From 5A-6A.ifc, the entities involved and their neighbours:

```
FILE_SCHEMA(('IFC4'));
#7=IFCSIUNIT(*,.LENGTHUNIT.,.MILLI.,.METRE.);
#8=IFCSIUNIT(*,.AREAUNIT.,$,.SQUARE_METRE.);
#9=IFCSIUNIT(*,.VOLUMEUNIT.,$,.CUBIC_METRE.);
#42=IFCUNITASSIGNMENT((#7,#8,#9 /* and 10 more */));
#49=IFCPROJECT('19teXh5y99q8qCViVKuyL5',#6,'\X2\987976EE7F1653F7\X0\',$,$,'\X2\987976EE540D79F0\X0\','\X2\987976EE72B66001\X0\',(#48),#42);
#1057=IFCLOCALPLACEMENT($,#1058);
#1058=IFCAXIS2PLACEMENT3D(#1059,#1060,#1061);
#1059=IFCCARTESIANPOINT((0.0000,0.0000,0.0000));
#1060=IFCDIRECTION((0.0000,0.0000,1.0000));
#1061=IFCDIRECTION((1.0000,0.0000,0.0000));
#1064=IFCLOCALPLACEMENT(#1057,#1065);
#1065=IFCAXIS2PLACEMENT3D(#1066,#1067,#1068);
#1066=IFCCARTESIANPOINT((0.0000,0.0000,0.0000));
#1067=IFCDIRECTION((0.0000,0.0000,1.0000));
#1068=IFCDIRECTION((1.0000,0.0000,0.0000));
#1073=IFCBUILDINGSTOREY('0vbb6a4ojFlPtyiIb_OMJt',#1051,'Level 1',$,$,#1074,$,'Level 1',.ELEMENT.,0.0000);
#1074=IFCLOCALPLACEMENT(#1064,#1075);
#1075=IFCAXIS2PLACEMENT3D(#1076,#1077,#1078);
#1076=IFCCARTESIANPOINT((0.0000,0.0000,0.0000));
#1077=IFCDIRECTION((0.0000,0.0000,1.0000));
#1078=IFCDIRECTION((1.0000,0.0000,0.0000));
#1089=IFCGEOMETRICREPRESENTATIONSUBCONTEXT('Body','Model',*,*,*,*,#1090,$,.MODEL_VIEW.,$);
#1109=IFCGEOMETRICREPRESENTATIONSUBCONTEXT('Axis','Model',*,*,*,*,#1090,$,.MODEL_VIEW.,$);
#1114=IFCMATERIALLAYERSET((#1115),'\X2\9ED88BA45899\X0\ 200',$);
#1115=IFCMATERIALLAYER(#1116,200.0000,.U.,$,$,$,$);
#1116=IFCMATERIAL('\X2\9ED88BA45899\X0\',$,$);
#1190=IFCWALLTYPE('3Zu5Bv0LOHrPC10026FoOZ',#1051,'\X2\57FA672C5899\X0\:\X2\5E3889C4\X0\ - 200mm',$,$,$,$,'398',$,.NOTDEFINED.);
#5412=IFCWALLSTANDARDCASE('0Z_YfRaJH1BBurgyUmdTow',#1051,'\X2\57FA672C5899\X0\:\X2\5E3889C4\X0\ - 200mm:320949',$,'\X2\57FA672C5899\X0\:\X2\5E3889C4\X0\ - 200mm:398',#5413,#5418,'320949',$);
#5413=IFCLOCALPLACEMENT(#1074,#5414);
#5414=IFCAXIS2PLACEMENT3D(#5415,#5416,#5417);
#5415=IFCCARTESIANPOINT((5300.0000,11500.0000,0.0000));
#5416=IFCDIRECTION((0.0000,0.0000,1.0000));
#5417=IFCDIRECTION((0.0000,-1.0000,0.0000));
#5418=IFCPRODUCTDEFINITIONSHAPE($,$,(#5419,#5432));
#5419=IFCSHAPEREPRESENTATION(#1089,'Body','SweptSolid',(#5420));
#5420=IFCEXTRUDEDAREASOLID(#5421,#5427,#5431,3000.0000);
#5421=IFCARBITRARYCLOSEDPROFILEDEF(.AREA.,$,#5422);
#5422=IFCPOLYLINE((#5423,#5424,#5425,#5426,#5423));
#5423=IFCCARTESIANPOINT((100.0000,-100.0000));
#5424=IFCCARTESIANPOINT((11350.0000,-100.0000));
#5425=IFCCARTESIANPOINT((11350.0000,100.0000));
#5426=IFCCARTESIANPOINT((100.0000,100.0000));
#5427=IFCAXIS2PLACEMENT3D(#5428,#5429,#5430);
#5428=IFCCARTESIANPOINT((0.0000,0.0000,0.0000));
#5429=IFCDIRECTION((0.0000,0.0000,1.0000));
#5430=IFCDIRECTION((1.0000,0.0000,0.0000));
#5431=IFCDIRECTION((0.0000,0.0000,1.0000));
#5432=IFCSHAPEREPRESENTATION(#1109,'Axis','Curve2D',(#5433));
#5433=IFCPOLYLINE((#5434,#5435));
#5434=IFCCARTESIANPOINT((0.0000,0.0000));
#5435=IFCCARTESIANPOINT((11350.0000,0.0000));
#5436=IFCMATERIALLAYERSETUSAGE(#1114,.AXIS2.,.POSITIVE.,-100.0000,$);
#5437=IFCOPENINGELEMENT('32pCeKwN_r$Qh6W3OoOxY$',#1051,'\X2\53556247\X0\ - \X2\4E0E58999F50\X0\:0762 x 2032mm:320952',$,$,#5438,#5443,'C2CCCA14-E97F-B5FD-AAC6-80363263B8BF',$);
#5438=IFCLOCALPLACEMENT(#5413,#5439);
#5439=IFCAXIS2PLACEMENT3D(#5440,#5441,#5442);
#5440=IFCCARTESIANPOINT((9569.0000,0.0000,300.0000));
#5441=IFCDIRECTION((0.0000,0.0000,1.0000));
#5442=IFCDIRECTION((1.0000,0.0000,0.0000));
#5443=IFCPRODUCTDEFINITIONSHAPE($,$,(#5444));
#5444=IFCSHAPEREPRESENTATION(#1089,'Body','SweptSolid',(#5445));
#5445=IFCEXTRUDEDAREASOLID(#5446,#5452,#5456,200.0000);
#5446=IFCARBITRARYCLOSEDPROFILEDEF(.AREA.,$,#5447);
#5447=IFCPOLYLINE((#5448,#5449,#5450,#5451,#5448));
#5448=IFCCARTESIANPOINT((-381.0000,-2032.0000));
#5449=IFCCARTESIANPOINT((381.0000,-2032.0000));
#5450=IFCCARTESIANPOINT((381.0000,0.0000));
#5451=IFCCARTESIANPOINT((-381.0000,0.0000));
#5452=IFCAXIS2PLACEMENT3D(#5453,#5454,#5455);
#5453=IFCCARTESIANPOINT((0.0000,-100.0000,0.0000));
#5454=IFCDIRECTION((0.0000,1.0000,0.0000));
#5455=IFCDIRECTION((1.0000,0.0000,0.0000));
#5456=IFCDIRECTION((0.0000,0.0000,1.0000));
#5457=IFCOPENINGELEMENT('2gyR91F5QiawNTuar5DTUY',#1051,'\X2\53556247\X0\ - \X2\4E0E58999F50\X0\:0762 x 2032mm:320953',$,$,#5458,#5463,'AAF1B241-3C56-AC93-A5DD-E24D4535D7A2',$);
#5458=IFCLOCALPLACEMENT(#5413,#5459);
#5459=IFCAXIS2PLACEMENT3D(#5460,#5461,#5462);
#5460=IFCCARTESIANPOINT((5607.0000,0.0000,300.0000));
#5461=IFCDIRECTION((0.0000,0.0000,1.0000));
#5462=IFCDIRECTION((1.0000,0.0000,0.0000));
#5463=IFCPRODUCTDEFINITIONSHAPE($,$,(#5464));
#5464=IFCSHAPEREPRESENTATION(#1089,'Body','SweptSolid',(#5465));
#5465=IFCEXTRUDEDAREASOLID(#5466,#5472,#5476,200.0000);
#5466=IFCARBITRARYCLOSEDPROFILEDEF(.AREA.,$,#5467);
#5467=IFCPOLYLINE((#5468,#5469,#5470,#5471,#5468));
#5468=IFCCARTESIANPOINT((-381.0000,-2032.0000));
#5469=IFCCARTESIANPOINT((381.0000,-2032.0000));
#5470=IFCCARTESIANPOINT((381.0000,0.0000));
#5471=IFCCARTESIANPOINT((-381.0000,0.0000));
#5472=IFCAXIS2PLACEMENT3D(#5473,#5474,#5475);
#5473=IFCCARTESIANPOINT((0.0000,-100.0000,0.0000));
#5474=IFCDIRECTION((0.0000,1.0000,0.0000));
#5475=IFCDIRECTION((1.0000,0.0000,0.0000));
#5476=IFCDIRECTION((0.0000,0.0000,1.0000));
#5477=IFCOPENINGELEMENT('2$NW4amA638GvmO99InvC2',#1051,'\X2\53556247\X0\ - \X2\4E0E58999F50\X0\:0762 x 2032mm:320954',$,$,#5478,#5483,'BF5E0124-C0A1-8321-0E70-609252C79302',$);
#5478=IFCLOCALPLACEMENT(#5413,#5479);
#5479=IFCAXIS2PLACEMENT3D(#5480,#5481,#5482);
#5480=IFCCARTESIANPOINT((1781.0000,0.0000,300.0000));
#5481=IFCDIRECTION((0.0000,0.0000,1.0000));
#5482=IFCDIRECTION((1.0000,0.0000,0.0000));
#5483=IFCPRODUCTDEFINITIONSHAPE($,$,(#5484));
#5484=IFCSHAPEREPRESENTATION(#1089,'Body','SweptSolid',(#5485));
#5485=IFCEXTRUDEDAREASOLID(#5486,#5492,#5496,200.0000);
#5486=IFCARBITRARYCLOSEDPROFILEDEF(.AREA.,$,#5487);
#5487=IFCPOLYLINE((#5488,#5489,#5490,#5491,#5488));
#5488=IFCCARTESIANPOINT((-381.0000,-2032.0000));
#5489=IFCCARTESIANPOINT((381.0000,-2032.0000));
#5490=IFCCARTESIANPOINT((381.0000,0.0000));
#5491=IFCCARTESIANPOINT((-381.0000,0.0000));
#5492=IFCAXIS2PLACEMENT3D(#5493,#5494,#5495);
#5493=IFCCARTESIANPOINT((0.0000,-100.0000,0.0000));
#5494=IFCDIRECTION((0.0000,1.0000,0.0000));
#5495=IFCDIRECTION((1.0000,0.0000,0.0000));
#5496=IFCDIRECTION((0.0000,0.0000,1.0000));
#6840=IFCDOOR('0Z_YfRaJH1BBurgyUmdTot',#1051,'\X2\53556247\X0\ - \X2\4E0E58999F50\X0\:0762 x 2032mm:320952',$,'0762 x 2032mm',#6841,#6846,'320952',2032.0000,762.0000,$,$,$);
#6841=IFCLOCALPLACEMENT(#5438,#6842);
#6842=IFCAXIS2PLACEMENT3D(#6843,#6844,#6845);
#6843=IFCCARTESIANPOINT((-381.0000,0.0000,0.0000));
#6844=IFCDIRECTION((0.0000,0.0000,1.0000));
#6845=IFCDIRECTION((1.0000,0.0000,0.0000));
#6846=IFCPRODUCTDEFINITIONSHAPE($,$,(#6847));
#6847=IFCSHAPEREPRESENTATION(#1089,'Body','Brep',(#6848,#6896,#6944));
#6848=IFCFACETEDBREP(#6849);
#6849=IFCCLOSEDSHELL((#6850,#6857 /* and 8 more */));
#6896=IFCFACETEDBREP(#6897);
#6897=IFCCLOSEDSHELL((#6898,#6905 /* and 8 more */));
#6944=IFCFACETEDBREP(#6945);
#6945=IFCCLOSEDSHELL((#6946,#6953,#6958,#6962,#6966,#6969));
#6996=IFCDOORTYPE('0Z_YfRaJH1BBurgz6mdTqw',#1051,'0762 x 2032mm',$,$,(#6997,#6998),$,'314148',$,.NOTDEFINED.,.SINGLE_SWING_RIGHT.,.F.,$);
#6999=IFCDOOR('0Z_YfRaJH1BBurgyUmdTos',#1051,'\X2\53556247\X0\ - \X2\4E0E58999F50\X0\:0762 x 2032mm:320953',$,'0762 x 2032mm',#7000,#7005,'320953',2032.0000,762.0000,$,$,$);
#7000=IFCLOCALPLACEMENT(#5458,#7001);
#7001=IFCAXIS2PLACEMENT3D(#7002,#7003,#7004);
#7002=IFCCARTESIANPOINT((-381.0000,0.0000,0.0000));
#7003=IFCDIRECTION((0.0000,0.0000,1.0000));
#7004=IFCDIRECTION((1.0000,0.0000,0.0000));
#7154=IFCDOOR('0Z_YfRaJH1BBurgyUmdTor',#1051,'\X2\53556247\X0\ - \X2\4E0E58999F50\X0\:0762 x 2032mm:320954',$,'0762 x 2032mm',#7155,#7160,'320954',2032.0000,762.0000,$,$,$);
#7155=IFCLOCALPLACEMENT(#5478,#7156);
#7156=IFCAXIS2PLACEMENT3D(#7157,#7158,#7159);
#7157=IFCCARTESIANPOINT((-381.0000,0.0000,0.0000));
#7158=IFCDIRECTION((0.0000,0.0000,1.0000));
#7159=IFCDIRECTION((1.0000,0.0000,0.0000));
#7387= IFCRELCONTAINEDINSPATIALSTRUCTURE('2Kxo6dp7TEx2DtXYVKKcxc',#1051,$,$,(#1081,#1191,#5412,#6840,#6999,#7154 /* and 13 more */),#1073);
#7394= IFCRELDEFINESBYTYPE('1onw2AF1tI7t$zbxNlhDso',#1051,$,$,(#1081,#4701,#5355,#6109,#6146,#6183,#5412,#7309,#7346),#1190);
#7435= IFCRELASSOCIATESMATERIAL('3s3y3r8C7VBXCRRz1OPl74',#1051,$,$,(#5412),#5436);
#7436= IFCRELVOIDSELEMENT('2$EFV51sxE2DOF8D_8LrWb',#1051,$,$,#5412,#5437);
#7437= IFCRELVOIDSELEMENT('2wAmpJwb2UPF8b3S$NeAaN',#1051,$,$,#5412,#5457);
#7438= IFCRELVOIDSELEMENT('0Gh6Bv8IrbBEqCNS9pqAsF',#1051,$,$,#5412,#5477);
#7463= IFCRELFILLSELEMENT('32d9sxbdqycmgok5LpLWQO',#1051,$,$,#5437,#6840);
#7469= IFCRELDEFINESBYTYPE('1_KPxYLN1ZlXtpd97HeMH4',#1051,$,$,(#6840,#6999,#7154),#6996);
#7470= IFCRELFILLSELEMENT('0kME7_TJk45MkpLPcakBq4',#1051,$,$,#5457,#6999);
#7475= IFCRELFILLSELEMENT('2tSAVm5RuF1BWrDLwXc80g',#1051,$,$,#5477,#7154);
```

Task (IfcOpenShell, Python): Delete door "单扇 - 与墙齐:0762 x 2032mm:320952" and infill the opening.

```python
import ifcopenshell
import ifcopenshell.api.feature
import ifcopenshell.api.root
import ifcopenshell.geom
import ifcopenshell.util.shape

model = ifcopenshell.open("5A-6A.ifc")
settings = ifcopenshell.geom.settings()


def volume(element):
    """Net volume in cubic metres, openings subtracted."""
    shape = ifcopenshell.geom.create_shape(settings, element)
    return ifcopenshell.util.shape.get_volume(shape.geometry)


door = model.by_guid("0Z_YfRaJH1BBurgyUmdTot")
opening = door.FillsVoids[0].RelatingOpeningElement
wall = opening.VoidsElements[0].RelatingBuildingElement
before = volume(wall)

ifcopenshell.api.root.remove_product(model, product=door)
ifcopenshell.api.feature.remove_feature(model, feature=opening)

after = volume(wall)

print(f"wall volume {before:.3f} -> {after:.3f} m3")

model.write("5A-6A-out.ifc")
```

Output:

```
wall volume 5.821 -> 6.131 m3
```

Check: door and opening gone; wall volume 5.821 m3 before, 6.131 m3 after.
